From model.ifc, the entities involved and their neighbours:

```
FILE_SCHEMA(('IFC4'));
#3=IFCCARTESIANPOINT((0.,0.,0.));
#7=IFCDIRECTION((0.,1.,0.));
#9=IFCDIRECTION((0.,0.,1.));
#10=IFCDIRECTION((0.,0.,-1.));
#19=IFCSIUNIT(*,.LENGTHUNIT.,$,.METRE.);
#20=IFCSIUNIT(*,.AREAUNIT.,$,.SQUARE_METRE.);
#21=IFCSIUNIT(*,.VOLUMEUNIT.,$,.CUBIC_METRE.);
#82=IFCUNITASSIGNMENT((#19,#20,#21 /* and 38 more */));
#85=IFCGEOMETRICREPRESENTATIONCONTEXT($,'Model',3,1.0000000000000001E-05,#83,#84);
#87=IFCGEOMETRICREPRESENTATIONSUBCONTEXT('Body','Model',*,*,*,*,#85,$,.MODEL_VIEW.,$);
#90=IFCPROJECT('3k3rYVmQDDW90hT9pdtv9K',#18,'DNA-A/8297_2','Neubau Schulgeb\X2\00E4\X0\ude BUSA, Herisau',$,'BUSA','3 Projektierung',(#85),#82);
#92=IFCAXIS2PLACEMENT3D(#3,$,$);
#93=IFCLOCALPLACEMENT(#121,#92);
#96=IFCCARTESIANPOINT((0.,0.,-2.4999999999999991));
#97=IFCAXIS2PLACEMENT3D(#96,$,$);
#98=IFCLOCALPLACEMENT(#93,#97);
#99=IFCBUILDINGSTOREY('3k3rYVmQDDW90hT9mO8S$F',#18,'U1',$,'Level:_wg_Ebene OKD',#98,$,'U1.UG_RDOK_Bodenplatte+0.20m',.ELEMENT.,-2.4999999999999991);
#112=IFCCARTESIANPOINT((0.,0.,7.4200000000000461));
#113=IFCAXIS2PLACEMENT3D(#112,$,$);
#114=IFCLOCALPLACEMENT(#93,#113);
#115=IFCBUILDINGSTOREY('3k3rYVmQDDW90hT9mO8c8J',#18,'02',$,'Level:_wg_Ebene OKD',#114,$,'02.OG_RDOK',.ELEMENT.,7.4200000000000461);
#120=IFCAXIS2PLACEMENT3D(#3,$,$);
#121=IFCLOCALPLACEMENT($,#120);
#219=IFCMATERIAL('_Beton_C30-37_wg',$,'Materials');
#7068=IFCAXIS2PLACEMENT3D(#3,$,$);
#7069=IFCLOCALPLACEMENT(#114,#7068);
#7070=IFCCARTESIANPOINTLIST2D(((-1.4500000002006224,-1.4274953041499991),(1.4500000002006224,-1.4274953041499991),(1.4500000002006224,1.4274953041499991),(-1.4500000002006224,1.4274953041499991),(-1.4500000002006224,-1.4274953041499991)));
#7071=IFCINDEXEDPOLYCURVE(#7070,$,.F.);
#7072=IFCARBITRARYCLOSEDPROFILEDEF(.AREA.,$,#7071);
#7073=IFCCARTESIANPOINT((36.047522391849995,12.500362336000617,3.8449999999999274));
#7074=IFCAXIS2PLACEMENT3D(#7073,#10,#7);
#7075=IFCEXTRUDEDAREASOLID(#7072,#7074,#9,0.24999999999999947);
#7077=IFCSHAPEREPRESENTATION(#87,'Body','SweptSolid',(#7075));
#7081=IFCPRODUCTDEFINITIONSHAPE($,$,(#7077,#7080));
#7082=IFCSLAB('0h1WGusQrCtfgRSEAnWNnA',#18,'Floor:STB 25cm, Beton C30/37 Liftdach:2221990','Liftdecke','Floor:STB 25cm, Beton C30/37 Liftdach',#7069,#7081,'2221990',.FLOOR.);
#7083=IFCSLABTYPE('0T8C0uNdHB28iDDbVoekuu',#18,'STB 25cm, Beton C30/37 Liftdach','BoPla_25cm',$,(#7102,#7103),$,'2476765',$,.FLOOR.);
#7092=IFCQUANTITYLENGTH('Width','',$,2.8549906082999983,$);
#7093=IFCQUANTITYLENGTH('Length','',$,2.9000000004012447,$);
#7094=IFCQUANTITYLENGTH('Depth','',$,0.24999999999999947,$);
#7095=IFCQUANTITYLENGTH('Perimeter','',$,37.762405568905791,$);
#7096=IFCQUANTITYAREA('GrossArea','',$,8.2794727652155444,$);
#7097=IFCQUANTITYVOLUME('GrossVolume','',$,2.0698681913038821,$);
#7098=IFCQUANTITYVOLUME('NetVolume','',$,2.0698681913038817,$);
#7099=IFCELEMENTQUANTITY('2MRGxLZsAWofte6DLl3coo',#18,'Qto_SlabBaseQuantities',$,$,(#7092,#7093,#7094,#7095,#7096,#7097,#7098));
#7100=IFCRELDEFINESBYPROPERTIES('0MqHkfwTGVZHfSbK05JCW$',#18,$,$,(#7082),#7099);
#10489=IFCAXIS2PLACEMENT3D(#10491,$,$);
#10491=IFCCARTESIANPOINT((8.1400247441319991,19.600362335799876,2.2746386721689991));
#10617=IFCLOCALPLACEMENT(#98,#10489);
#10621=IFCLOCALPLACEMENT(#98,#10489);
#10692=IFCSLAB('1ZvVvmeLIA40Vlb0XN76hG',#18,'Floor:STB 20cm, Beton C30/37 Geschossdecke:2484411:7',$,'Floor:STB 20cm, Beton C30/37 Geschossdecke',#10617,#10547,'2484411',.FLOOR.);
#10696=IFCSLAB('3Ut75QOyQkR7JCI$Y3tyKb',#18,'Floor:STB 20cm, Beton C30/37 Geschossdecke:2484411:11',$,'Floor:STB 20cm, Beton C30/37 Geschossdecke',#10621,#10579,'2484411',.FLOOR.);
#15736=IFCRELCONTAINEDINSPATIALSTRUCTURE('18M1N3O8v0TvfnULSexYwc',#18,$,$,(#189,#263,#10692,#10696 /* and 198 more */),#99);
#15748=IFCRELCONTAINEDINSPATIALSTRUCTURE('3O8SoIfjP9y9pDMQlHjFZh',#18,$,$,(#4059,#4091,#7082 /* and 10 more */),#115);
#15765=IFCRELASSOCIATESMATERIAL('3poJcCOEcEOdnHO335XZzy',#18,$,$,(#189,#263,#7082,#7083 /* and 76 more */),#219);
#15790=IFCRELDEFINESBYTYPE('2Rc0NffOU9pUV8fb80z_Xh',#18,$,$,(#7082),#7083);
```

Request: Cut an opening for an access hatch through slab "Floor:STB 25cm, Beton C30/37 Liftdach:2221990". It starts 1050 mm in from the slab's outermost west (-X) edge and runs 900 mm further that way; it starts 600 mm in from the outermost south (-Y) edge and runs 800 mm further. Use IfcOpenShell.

```python
import numpy as np
import ifcopenshell
import ifcopenshell.api.feature
import ifcopenshell.api.geometry
import ifcopenshell.api.pset
import ifcopenshell.api.root
import ifcopenshell.geom
import ifcopenshell.util.element
import ifcopenshell.util.placement
import ifcopenshell.util.representation
import ifcopenshell.util.shape
import ifcopenshell.util.unit

model = ifcopenshell.open("model.ifc")
unit_scale = ifcopenshell.util.unit.calculate_unit_scale(model)
volume_scale = ifcopenshell.util.unit.calculate_unit_scale(model, "VOLUMEUNIT")
settings = ifcopenshell.geom.settings()


def volume(element):
    """Net volume in cubic metres, openings subtracted."""
    shape = ifcopenshell.geom.create_shape(settings, element)
    return ifcopenshell.util.shape.get_volume(shape.geometry)


slab = model.by_guid("0h1WGusQrCtfgRSEAnWNnA")
before = volume(slab)

# Extent in the slab's own axes, in metres. The edges named are its -X and -Y sides.
slab_shape = ifcopenshell.geom.create_shape(settings, slab)
vertices = ifcopenshell.util.shape.get_vertices(slab_shape.geometry)
x_min, y_min, bottom = vertices.min(axis=0)
top = vertices[:, 2].max()

opening = ifcopenshell.api.root.create_entity(model, ifc_class="IfcOpeningElement", name="Access hatch opening", predefined_type="OPENING")
context = ifcopenshell.util.representation.get_context(model, "Model", "Body", "MODEL_VIEW")
width, depth = 0.9, 0.8
outline = [(0.0, 0.0), (width, 0.0), (width, depth), (0.0, depth), (0.0, 0.0)]
# Overshoot both faces by 50 mm so the cut is clean.
shape = ifcopenshell.api.geometry.add_slab_representation(
    model, context=context, depth=top - bottom + 0.1, polyline=outline
)
ifcopenshell.api.geometry.assign_representation(model, product=opening, representation=shape)

matrix = ifcopenshell.util.placement.get_local_placement(slab.ObjectPlacement)
matrix[:, 3] = matrix @ np.append(np.array([x_min + 1.05, y_min + 0.6, bottom - 0.05]) / unit_scale, 1.0)
ifcopenshell.api.geometry.edit_object_placement(model, product=opening, matrix=matrix, is_si=False)
ifcopenshell.api.feature.add_feature(model, feature=opening, element=slab)

after = volume(slab)

# Update the slab's stored quantities.
qto = model.by_id(ifcopenshell.util.element.get_pset(slab, "Qto_SlabBaseQuantities", should_inherit=False)["id"])
ifcopenshell.api.pset.edit_qto(model, qto=qto, properties={"NetVolume": after / volume_scale})

print(f"slab volume {before:.3f} -> {after:.3f} m3")

model.write("model_rev.ifc")
```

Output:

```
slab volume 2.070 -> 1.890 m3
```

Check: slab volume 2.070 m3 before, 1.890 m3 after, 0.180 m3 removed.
